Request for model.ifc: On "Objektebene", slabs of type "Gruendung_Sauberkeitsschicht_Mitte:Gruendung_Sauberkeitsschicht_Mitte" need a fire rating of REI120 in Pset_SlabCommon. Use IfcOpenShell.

First a look at what the model holds.

```python
import ifcopenshell
import ifcopenshell.util.element

model = ifcopenshell.open("model.ifc")
print(model.schema)
storey = next(s for s in model.by_type("IfcBuildingStorey") if s.Name == "Objektebene")
slabs = [e for e in ifcopenshell.util.element.get_decomposition(storey) if e.is_a("IfcSlab")]
seen = {}
for e in slabs:
    element_type = ifcopenshell.util.element.get_type(e)
    key = (element_type.Name if element_type != e and element_type else None, ifcopenshell.util.element.get_pset(e, "Pset_SlabCommon", "FireRating"))
    seen[key] = seen.get(key, 0) + 1
for (name, value), count in sorted(seen.items(), key=str):
    print(count, "x", name, "|", value)
```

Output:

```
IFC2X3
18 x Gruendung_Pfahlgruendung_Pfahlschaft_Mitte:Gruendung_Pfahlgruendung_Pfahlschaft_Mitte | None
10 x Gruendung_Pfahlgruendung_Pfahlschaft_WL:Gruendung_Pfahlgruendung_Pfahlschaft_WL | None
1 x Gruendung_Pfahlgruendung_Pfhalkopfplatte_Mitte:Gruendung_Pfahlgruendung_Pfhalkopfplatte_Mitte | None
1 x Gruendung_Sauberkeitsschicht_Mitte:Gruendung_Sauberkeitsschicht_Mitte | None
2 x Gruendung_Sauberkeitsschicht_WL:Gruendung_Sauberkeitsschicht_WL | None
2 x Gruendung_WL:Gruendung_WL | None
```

```python
import ifcopenshell
import ifcopenshell.api.pset
import ifcopenshell.util.element

model = ifcopenshell.open("model.ifc")

storey = next(s for s in model.by_type("IfcBuildingStorey") if s.Name == "Objektebene")
slabs = [e for e in ifcopenshell.util.element.get_decomposition(storey) if e.is_a("IfcSlab")]

count = 0
for e in slabs:
    element_type = ifcopenshell.util.element.get_type(e)
    if element_type in (None, e) or element_type.Name != "Gruendung_Sauberkeitsschicht_Mitte:Gruendung_Sauberkeitsschicht_Mitte":
        continue
    # add_pset returns the element's existing set when there is one.
    pset = ifcopenshell.api.pset.add_pset(model, product=e, name="Pset_SlabCommon")
    ifcopenshell.api.pset.edit_pset(model, pset=pset, properties={"FireRating": "REI120"})
    count += 1

print(count, "slabs updated")

model.write("model_rev.ifc")
```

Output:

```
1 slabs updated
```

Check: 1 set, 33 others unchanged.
